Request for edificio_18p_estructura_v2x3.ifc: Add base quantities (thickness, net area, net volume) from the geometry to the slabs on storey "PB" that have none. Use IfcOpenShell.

First a look at what the model holds.

```python
import ifcopenshell
import ifcopenshell.util.element
import ifcopenshell.util.unit

model = ifcopenshell.open("edificio_18p_estructura_v2x3.ifc")
print(model.schema)
for unit_type in ("LENGTHUNIT", "AREAUNIT", "VOLUMEUNIT"):
    print(unit_type, ifcopenshell.util.unit.calculate_unit_scale(model, unit_type))
storey = next(s for s in model.by_type("IfcBuildingStorey") if s.Name == "PB")
slabs = [e for e in ifcopenshell.util.element.get_decomposition(storey) if e.is_a("IfcSlab")]
for e in sorted(slabs, key=lambda e: e.id()):
    print(e.id(), e.is_a(), e.Name, list(ifcopenshell.util.element.get_psets(e, qtos_only=True)), sep=" | ")
```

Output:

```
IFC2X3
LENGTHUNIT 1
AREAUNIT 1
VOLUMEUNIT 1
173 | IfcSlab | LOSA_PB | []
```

```python
import ifcopenshell
import ifcopenshell.api.pset
import ifcopenshell.geom
import ifcopenshell.util.element
import ifcopenshell.util.shape
import ifcopenshell.util.unit

model = ifcopenshell.open("edificio_18p_estructura_v2x3.ifc")
unit_scale = ifcopenshell.util.unit.calculate_unit_scale(model)
area_scale = ifcopenshell.util.unit.calculate_unit_scale(model, "AREAUNIT")
volume_scale = ifcopenshell.util.unit.calculate_unit_scale(model, "VOLUMEUNIT")
settings = ifcopenshell.geom.settings()

storey = next(s for s in model.by_type("IfcBuildingStorey") if s.Name == "PB")
slabs = [e for e in ifcopenshell.util.element.get_decomposition(storey) if e.is_a("IfcSlab")]

for e in sorted(slabs, key=lambda e: e.id()):
    if ifcopenshell.util.element.get_psets(e, qtos_only=True, should_inherit=False):
        continue
    # Geometry comes back in metres, in the element's own axes.
    shape = ifcopenshell.geom.create_shape(settings, e)
    values = {
        "Width": ifcopenshell.util.shape.get_z(shape.geometry) / unit_scale,
        "NetArea": ifcopenshell.util.shape.get_footprint_area(shape.geometry) / area_scale,
        "NetVolume": ifcopenshell.util.shape.get_volume(shape.geometry) / volume_scale,
    }
    qto = ifcopenshell.api.pset.add_qto(model, product=e, name="BaseQuantities")
    ifcopenshell.api.pset.edit_qto(model, qto=qto, properties=values)
    print(e.id(), {k: round(v, 3) for k, v in values.items()})

model.write("edificio_18p_estructura_v2x3_updated.ifc")
```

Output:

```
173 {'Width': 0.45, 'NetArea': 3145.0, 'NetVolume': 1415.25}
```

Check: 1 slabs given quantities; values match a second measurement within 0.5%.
